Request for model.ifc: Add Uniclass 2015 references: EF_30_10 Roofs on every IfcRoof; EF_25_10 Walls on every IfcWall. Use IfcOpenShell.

First a look at what the model holds.

```python
import ifcopenshell

model = ifcopenshell.open("model.ifc")
print(model.schema)
print("classifications:", [c.Name for c in model.by_type("IfcClassification")])
for ifc_class in ("IfcDoor", "IfcRoof", "IfcStair", "IfcWall", "IfcWindow"):
    print(ifc_class, len(model.by_type(ifc_class)))
```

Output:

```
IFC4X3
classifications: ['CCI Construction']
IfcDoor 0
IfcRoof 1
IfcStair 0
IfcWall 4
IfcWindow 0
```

```python
import ifcopenshell
import ifcopenshell.api.classification

model = ifcopenshell.open("model.ifc")

system = ifcopenshell.api.classification.add_classification(model, classification="Uniclass 2015")

codes = {
    "IfcRoof": ("EF_30_10", "Roofs"),
    "IfcWall": ("EF_25_10", "Walls"),
}
for ifc_class, (code, name) in codes.items():
    products = model.by_type(ifc_class)
    ifcopenshell.api.classification.add_reference(
        model, products=products, classification=system, identification=code, name=name
    )
    print(code, len(products))

model.write("model_updated.ifc")
```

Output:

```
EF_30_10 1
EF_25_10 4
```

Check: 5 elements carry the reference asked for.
